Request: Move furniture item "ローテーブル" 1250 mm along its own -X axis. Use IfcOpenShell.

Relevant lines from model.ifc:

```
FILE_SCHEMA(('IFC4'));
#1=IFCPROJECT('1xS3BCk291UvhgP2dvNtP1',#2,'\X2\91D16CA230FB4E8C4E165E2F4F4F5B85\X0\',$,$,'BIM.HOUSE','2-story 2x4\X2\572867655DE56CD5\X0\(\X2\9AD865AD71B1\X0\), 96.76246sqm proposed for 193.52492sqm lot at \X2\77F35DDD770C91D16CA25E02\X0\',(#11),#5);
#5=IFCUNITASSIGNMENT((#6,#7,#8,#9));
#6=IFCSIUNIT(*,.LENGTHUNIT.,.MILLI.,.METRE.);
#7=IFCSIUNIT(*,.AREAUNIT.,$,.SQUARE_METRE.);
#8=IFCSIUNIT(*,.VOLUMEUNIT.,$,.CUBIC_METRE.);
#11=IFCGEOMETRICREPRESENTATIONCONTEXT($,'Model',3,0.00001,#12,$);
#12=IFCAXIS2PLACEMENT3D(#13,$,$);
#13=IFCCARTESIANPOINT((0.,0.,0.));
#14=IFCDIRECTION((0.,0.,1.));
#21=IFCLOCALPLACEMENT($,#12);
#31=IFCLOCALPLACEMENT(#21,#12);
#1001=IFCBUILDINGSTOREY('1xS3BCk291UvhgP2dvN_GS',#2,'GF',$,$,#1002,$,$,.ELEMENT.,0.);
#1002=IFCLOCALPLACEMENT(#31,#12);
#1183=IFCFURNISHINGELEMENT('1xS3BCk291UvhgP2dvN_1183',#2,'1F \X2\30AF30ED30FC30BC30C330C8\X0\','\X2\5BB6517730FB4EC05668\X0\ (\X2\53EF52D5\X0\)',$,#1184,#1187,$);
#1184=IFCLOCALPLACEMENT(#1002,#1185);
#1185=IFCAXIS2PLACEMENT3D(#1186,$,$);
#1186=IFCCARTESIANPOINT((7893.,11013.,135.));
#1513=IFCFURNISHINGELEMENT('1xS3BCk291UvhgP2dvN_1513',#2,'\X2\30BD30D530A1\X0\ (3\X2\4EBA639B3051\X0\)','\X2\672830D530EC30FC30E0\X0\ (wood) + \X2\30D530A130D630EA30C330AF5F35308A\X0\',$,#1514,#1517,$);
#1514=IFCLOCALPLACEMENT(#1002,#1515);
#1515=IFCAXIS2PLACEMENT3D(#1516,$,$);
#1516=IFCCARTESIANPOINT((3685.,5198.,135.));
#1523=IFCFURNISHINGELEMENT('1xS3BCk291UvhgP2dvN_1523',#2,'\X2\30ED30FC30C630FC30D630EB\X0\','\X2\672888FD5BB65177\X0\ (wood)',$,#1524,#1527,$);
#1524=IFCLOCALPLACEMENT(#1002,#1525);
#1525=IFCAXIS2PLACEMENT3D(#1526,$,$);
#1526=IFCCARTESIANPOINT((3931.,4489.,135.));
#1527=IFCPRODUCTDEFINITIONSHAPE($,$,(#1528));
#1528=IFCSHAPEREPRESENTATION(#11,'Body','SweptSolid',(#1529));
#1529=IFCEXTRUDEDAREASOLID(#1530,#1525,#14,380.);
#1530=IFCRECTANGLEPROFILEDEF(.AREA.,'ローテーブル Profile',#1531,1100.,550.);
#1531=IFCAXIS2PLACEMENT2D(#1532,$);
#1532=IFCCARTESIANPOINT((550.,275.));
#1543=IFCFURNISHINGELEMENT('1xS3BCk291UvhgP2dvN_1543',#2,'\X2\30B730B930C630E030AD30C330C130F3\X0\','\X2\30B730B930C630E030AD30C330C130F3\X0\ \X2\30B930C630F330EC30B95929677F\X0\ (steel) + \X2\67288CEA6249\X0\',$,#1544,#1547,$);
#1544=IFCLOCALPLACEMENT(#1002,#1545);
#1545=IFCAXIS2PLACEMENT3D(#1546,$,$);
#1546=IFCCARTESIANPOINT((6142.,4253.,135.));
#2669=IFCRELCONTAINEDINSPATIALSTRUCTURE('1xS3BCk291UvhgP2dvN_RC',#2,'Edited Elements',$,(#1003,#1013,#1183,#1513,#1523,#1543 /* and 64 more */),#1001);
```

```python
import ifcopenshell
import ifcopenshell.api.geometry
import ifcopenshell.util.placement

model = ifcopenshell.open("model.ifc")

item = model.by_guid("1xS3BCk291UvhgP2dvN_1523")
matrix = ifcopenshell.util.placement.get_local_placement(item.ObjectPlacement)
matrix[:3, 3] -= matrix[:3, 0] * 1250.0
ifcopenshell.api.geometry.edit_object_placement(model, product=item, matrix=matrix, is_si=False)

print(ifcopenshell.util.placement.get_local_placement(item.ObjectPlacement).round(3) + 0.0)

model.write("model_updated.ifc")
```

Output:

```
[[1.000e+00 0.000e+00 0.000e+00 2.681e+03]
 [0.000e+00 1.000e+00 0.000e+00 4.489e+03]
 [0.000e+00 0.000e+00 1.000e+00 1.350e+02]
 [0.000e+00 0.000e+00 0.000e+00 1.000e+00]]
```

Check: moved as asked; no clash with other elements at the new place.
